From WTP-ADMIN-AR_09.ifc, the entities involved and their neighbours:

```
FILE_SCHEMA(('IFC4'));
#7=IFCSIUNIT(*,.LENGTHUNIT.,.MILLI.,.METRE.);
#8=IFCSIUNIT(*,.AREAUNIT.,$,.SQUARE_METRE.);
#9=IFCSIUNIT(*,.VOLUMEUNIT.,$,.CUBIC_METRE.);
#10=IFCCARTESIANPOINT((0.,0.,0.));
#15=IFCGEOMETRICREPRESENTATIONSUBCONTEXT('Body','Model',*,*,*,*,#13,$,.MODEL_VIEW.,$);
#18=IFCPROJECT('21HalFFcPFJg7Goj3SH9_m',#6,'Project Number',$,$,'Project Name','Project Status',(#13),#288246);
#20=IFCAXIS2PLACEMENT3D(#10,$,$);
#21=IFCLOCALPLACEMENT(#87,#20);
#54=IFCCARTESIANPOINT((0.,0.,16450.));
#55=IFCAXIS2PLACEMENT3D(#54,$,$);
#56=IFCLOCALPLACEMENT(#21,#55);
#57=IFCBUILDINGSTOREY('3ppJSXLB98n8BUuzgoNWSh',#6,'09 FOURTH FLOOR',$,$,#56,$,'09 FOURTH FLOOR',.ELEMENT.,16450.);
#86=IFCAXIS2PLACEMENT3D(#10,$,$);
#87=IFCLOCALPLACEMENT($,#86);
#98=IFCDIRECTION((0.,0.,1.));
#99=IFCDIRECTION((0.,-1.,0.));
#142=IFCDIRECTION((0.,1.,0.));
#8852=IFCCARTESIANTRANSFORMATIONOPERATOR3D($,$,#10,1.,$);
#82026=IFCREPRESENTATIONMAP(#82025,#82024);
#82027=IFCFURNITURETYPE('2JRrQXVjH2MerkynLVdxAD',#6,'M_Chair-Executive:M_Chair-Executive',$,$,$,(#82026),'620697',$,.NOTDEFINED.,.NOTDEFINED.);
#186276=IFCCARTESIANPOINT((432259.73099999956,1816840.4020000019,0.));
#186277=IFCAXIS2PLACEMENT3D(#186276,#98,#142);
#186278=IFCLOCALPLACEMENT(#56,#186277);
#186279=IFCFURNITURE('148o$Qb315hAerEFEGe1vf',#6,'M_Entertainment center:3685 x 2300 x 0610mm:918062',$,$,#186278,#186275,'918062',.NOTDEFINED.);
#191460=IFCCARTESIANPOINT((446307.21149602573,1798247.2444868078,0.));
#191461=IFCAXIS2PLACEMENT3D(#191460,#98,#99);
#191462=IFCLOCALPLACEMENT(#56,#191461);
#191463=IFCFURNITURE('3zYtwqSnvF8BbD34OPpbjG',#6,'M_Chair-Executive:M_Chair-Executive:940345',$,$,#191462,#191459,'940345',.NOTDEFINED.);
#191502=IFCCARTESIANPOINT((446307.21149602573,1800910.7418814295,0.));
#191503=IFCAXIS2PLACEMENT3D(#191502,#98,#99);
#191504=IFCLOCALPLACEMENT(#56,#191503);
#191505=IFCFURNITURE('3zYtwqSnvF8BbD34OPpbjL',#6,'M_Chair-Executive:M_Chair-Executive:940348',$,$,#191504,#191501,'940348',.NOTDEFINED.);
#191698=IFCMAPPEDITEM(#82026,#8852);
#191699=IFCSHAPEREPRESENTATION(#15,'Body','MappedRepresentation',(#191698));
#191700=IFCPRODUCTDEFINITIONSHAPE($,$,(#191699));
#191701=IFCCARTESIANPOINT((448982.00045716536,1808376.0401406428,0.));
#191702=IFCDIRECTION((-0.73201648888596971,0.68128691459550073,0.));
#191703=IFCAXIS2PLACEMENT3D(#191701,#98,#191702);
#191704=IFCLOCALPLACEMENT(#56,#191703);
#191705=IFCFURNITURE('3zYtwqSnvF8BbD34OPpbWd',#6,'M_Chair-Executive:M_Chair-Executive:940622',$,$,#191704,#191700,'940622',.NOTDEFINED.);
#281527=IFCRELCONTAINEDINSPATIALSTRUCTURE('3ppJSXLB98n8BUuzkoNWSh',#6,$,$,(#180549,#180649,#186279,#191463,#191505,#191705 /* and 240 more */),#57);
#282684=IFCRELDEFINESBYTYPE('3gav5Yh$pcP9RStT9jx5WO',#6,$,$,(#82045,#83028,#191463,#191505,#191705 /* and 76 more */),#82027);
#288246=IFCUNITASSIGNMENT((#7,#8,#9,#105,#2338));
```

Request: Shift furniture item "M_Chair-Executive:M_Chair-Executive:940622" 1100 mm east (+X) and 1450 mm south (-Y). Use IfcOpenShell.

```python
import ifcopenshell
import ifcopenshell.api.geometry
import ifcopenshell.util.placement

model = ifcopenshell.open("WTP-ADMIN-AR_09.ifc")

item = model.by_guid("3zYtwqSnvF8BbD34OPpbWd")
matrix = ifcopenshell.util.placement.get_local_placement(item.ObjectPlacement)
matrix[0, 3] += 1100.0
matrix[1, 3] -= 1450.0
ifcopenshell.api.geometry.edit_object_placement(model, product=item, matrix=matrix, is_si=False)

print(ifcopenshell.util.placement.get_local_placement(item.ObjectPlacement).round(3) + 0.0)

model.write("WTP-ADMIN-AR_09_rev.ifc")
```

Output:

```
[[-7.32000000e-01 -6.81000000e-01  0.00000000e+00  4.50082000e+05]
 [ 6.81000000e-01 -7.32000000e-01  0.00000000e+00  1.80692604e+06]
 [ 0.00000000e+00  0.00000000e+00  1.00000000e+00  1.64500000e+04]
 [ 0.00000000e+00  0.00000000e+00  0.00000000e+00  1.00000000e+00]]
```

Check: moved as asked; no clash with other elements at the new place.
